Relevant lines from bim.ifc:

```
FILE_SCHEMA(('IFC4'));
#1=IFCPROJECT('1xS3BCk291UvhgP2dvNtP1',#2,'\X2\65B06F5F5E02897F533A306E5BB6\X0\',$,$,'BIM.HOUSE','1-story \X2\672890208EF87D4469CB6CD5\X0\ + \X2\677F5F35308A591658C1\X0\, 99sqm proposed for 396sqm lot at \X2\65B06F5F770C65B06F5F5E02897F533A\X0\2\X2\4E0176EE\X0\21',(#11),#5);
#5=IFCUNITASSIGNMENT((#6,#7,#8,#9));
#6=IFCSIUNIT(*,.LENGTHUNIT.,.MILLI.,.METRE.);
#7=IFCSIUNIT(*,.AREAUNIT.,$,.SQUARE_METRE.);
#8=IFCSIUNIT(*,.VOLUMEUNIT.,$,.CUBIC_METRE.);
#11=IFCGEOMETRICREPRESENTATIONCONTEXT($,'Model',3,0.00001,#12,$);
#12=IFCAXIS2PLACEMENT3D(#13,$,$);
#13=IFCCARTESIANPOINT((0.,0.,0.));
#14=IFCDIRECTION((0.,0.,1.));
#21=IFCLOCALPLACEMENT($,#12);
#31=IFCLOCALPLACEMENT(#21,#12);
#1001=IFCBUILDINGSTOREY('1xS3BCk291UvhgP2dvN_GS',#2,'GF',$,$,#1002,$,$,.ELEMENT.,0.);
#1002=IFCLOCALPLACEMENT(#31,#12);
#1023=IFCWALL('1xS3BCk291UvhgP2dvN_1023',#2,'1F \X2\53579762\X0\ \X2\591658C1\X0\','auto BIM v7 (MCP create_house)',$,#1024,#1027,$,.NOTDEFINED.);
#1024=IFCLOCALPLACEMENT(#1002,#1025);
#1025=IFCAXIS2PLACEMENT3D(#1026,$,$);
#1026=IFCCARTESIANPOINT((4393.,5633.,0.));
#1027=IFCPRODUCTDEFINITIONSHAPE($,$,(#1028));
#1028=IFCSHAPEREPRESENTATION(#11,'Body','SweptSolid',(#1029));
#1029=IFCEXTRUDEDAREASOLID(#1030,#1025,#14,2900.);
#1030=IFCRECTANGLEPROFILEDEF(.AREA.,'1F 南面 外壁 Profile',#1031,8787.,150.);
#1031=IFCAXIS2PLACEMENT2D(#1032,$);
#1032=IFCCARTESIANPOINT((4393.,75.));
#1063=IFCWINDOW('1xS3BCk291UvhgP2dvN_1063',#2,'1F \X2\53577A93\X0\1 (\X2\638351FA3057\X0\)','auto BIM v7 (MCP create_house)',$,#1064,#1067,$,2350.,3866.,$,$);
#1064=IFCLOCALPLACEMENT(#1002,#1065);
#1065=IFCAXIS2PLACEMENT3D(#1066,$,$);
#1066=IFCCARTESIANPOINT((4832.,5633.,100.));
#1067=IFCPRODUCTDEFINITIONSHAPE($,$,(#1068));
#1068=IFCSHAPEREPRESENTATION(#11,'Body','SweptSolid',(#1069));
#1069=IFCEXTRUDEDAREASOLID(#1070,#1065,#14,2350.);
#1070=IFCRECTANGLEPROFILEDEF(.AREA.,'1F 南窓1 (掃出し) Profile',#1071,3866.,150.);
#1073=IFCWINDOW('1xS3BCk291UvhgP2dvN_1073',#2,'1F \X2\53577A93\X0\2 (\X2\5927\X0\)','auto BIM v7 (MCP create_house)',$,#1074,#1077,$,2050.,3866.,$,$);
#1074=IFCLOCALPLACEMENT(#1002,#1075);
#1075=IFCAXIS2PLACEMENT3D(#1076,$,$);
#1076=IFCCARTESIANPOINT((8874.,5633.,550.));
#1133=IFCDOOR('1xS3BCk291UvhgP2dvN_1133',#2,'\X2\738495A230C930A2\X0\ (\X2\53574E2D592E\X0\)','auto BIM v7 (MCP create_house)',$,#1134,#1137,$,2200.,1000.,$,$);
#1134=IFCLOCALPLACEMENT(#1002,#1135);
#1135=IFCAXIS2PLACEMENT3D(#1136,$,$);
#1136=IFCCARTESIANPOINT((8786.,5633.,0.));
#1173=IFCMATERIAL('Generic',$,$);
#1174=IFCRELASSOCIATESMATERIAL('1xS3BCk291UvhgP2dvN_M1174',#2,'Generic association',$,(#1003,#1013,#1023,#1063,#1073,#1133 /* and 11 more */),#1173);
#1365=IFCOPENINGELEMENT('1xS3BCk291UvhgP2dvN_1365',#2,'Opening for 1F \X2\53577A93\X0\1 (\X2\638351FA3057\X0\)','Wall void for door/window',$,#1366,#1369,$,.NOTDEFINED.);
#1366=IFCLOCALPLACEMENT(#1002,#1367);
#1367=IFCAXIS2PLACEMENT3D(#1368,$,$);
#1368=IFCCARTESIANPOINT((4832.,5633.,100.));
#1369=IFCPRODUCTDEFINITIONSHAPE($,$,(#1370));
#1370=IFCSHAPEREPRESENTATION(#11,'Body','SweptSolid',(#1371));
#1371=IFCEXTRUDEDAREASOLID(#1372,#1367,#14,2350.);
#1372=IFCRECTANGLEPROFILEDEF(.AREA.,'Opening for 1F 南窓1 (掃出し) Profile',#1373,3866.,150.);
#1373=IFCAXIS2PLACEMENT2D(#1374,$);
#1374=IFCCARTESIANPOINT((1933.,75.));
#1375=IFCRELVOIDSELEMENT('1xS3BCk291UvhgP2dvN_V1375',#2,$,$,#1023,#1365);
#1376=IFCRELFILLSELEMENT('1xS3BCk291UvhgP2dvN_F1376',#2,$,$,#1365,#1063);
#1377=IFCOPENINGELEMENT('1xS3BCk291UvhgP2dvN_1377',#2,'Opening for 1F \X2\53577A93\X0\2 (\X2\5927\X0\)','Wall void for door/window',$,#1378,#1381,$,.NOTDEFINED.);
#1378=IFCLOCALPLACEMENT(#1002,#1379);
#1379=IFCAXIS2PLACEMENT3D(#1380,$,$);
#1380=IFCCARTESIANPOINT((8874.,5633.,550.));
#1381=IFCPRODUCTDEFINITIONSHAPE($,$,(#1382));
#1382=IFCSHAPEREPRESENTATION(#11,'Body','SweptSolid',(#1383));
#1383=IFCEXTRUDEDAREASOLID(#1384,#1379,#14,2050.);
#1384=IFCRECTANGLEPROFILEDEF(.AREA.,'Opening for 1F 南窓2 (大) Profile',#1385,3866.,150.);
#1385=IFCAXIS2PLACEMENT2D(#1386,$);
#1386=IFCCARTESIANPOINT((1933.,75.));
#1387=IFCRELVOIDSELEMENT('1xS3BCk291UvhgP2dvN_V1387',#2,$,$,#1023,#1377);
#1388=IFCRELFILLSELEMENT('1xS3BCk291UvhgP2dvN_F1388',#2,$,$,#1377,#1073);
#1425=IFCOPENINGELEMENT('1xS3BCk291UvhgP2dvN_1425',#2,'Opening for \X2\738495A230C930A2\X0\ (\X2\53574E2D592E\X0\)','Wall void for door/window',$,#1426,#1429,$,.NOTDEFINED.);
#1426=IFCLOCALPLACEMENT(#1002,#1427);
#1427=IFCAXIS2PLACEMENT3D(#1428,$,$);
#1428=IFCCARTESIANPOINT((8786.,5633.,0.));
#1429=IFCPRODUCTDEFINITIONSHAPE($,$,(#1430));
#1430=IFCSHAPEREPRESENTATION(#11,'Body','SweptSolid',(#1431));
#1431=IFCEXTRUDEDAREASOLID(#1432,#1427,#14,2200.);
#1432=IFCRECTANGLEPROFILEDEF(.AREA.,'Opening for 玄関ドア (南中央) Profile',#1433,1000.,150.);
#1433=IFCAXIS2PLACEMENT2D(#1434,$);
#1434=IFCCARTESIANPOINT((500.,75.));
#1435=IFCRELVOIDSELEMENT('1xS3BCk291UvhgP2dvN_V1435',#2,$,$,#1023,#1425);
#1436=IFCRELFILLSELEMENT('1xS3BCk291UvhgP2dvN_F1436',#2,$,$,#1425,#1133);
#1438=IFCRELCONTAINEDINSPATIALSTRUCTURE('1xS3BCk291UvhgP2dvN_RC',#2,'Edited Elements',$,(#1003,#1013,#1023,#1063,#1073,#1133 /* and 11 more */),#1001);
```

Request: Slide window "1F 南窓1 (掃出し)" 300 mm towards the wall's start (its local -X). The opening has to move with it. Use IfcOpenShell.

```python
import ifcopenshell
import ifcopenshell.api.geometry
import ifcopenshell.util.placement

model = ifcopenshell.open("bim.ifc")

window = model.by_id(1063)
opening = window.FillsVoids[0].RelatingOpeningElement
wall = opening.VoidsElements[0].RelatingBuildingElement

wall_matrix = ifcopenshell.util.placement.get_local_placement(wall.ObjectPlacement)
shift = wall_matrix[:3, 0] * -300.0
before = ifcopenshell.util.placement.get_local_placement(window.ObjectPlacement)[:3, 3].copy()

# The window is not placed relative to its opening, so move both.
for product in (opening, window):
    matrix = ifcopenshell.util.placement.get_local_placement(product.ObjectPlacement)
    matrix[:3, 3] += shift
    ifcopenshell.api.geometry.edit_object_placement(model, product=product, matrix=matrix, is_si=False)

after = ifcopenshell.util.placement.get_local_placement(window.ObjectPlacement)[:3, 3]
print("window moved by", (after - before).round(3) + 0.0)

model.write("bim_rev.ifc")
```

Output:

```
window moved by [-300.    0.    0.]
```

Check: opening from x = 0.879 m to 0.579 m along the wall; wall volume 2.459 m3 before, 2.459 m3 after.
